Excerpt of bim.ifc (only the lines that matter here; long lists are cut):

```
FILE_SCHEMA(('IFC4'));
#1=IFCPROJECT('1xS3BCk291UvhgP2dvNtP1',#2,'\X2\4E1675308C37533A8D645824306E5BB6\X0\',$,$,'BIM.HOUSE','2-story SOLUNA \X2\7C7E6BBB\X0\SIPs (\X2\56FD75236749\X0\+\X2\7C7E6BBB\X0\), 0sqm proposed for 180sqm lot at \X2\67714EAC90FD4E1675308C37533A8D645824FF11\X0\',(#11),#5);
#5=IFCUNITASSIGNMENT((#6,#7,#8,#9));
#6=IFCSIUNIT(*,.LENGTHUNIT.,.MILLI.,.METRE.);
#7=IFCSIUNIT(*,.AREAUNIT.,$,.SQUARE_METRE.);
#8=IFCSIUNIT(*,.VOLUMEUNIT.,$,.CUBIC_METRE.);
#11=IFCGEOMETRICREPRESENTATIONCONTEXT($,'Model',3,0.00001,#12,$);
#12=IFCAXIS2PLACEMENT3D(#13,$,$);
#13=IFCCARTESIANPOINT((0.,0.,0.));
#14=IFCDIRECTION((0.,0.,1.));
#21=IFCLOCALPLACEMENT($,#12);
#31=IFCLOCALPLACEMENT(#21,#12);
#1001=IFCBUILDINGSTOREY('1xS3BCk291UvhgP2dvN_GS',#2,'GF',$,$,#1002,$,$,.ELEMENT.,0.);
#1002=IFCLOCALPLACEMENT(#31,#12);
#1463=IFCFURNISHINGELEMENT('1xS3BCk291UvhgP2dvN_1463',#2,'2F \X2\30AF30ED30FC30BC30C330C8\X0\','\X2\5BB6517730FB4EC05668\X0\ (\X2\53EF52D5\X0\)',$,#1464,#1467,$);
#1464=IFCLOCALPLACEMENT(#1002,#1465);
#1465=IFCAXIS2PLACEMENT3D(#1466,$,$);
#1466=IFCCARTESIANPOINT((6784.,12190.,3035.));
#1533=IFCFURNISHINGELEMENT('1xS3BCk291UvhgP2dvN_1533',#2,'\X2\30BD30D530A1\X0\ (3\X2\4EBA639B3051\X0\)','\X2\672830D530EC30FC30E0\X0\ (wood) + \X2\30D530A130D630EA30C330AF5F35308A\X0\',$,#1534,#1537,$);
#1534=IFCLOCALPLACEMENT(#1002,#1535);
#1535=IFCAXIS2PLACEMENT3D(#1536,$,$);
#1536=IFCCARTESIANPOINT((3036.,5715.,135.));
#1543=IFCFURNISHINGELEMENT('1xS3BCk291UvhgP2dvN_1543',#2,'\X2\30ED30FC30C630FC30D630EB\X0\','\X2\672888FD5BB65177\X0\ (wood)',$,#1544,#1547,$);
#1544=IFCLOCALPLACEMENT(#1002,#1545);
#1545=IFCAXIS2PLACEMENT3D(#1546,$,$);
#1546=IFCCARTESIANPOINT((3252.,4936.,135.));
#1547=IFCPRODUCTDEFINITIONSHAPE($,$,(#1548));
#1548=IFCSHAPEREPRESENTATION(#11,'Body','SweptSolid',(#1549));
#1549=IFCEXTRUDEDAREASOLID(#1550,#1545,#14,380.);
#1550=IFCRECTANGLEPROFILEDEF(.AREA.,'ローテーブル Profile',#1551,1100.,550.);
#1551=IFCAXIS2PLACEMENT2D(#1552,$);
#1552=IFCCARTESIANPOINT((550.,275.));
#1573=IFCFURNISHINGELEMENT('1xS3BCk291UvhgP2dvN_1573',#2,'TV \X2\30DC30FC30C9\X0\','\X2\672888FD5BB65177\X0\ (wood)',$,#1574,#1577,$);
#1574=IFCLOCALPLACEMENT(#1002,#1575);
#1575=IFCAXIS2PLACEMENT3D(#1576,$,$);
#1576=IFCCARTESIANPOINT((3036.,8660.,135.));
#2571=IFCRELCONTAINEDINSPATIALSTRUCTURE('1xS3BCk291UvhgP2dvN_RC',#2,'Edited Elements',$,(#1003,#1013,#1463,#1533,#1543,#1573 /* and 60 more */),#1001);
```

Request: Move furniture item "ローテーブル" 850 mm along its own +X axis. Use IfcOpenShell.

```python
import ifcopenshell
import ifcopenshell.api.geometry
import ifcopenshell.util.placement
import ifcopenshell.util.unit

model = ifcopenshell.open("bim.ifc")
unit_scale = ifcopenshell.util.unit.calculate_unit_scale(model)

item = model.by_guid("1xS3BCk291UvhgP2dvN_1543")
matrix = ifcopenshell.util.placement.get_local_placement(item.ObjectPlacement)
matrix[:3, 3] += matrix[:3, 0] * 0.85 / unit_scale
ifcopenshell.api.geometry.edit_object_placement(model, product=item, matrix=matrix, is_si=False)

print(ifcopenshell.util.placement.get_local_placement(item.ObjectPlacement).round(3) + 0.0)

model.write("bim_v2.ifc")
```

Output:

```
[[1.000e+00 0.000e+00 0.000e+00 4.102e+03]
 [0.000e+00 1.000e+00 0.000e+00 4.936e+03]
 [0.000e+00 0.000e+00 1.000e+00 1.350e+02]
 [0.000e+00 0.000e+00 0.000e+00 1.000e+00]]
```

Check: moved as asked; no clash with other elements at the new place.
